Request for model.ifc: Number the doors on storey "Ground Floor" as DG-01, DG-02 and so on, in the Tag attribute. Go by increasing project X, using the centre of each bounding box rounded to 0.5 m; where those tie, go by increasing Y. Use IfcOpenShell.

First a look at what the model holds.

```python
import ifcopenshell
import ifcopenshell.util.element
import ifcopenshell.util.placement

model = ifcopenshell.open("model.ifc")
print(model.schema)
storey = next(s for s in model.by_type("IfcBuildingStorey") if s.Name == "Ground Floor")
doors = [e for e in ifcopenshell.util.element.get_decomposition(storey) if e.is_a("IfcDoor")]
for e in sorted(doors, key=lambda e: e.id()):
    origin = ifcopenshell.util.placement.get_local_placement(e.ObjectPlacement)[:3, 3]
    print(e.id(), e.Tag, e.Name, origin.round(2) + 0.0, sep=" | ")
```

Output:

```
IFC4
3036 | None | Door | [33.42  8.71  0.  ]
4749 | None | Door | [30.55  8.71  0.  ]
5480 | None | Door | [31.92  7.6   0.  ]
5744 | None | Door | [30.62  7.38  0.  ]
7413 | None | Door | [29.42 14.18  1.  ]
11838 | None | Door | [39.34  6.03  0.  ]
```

```python
import ifcopenshell
import ifcopenshell.geom
import ifcopenshell.util.element
import ifcopenshell.util.shape

model = ifcopenshell.open("model.ifc")
settings = ifcopenshell.geom.settings()
settings.set("use-world-coords", True)


def centre(element):
    shape = ifcopenshell.geom.create_shape(settings, element)
    return ifcopenshell.util.shape.get_bbox_centroid(shape.geometry)


storey = next(s for s in model.by_type("IfcBuildingStorey") if s.Name == "Ground Floor")
doors = [e for e in ifcopenshell.util.element.get_decomposition(storey) if e.is_a("IfcDoor")]

# Insertion points can sit at a corner or the storey origin, so sort by the geometry (in metres).
centres = {e: centre(e) for e in doors}
doors.sort(key=lambda e: (round(centres[e][0] / 0.5), centres[e][1]))

for i, e in enumerate(doors, start=1):
    number = f"DG-{i:02d}"
    e.Tag = number
    print(e.id(), number)

model.write("model_v2.ifc")
```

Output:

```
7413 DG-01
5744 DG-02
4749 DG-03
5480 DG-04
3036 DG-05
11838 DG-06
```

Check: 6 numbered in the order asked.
